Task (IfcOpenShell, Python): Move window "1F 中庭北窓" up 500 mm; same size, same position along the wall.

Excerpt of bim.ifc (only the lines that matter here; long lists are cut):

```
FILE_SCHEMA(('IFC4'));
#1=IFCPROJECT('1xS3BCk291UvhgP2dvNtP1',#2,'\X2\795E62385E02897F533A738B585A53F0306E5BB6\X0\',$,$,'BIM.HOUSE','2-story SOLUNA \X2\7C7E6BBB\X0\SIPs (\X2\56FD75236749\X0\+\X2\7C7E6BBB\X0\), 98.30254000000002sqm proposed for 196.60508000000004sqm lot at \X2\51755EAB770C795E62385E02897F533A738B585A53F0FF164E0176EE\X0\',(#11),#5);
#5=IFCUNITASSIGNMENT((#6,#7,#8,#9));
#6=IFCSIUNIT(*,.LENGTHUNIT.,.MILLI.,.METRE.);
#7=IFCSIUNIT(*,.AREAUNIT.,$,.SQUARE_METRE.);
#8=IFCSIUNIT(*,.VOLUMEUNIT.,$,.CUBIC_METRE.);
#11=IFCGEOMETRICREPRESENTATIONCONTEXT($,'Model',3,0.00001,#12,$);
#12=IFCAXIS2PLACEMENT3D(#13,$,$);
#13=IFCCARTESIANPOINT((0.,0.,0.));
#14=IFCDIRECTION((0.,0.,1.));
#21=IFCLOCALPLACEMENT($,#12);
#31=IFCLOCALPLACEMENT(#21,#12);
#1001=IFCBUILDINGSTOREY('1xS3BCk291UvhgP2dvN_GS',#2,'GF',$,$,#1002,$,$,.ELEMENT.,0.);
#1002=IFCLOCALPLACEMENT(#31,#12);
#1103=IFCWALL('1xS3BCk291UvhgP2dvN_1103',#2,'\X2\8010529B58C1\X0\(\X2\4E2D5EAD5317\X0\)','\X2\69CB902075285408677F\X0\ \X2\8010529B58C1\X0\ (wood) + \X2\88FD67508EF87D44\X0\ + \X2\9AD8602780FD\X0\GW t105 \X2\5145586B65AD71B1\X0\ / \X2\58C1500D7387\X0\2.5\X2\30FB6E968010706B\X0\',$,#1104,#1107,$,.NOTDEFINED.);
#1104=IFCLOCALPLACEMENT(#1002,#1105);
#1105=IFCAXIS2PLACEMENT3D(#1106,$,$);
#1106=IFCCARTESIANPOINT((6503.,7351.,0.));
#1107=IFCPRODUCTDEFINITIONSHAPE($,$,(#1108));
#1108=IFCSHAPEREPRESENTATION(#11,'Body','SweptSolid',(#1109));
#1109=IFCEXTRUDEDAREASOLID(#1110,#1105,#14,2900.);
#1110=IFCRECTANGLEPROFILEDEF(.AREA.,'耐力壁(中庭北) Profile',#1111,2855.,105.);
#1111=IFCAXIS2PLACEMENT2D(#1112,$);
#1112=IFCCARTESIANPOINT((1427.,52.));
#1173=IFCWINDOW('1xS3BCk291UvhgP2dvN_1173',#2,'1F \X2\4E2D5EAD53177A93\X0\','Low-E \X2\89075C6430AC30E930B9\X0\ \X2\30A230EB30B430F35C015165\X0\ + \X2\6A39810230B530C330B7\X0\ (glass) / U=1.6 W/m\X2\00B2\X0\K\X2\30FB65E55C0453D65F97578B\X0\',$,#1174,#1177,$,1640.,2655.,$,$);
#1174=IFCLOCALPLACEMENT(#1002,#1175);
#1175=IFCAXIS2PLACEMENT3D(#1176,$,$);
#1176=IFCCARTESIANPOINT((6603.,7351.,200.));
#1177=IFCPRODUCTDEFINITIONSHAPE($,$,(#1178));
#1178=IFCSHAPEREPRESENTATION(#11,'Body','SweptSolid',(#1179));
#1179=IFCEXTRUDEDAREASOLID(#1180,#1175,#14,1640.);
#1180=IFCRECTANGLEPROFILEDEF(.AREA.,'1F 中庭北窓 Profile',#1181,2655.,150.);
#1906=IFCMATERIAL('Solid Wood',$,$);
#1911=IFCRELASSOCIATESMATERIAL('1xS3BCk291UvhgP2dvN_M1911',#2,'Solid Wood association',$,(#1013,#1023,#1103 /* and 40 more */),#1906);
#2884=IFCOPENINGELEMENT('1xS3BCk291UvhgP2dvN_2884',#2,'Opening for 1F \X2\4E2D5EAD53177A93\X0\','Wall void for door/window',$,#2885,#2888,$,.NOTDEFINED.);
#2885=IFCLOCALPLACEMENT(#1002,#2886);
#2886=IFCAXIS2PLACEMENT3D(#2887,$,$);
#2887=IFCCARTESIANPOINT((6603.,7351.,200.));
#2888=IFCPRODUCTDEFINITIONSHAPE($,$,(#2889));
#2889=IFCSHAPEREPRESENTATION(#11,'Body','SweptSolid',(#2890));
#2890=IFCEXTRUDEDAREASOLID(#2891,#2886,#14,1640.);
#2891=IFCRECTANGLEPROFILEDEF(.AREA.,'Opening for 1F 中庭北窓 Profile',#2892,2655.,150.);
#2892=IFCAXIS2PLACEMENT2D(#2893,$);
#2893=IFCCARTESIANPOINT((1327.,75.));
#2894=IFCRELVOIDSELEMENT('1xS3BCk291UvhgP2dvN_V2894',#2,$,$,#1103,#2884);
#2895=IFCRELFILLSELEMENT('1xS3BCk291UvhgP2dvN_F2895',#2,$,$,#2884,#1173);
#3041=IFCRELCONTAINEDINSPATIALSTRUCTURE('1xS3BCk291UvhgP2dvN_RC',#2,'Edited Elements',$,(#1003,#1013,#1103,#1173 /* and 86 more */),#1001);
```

```python
import numpy as np
import ifcopenshell
import ifcopenshell.api.geometry
import ifcopenshell.util.placement
import ifcopenshell.util.unit

model = ifcopenshell.open("bim.ifc")
unit_scale = ifcopenshell.util.unit.calculate_unit_scale(model)

window = model.by_guid("1xS3BCk291UvhgP2dvN_1173")
opening = window.FillsVoids[0].RelatingOpeningElement
dz = 500.0

shift = np.array([0.0, 0.0, dz])
# The window is not placed relative to its opening, so move both.
for product in (opening, window):
    matrix = ifcopenshell.util.placement.get_local_placement(product.ObjectPlacement)
    matrix[:3, 3] += shift
    ifcopenshell.api.geometry.edit_object_placement(model, product=product, matrix=matrix, is_si=False)

print(f"moved by {dz * unit_scale:+.3f} m")

model.write("bim_edited.ifc")
```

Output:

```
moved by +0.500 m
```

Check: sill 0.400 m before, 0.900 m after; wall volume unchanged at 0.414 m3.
